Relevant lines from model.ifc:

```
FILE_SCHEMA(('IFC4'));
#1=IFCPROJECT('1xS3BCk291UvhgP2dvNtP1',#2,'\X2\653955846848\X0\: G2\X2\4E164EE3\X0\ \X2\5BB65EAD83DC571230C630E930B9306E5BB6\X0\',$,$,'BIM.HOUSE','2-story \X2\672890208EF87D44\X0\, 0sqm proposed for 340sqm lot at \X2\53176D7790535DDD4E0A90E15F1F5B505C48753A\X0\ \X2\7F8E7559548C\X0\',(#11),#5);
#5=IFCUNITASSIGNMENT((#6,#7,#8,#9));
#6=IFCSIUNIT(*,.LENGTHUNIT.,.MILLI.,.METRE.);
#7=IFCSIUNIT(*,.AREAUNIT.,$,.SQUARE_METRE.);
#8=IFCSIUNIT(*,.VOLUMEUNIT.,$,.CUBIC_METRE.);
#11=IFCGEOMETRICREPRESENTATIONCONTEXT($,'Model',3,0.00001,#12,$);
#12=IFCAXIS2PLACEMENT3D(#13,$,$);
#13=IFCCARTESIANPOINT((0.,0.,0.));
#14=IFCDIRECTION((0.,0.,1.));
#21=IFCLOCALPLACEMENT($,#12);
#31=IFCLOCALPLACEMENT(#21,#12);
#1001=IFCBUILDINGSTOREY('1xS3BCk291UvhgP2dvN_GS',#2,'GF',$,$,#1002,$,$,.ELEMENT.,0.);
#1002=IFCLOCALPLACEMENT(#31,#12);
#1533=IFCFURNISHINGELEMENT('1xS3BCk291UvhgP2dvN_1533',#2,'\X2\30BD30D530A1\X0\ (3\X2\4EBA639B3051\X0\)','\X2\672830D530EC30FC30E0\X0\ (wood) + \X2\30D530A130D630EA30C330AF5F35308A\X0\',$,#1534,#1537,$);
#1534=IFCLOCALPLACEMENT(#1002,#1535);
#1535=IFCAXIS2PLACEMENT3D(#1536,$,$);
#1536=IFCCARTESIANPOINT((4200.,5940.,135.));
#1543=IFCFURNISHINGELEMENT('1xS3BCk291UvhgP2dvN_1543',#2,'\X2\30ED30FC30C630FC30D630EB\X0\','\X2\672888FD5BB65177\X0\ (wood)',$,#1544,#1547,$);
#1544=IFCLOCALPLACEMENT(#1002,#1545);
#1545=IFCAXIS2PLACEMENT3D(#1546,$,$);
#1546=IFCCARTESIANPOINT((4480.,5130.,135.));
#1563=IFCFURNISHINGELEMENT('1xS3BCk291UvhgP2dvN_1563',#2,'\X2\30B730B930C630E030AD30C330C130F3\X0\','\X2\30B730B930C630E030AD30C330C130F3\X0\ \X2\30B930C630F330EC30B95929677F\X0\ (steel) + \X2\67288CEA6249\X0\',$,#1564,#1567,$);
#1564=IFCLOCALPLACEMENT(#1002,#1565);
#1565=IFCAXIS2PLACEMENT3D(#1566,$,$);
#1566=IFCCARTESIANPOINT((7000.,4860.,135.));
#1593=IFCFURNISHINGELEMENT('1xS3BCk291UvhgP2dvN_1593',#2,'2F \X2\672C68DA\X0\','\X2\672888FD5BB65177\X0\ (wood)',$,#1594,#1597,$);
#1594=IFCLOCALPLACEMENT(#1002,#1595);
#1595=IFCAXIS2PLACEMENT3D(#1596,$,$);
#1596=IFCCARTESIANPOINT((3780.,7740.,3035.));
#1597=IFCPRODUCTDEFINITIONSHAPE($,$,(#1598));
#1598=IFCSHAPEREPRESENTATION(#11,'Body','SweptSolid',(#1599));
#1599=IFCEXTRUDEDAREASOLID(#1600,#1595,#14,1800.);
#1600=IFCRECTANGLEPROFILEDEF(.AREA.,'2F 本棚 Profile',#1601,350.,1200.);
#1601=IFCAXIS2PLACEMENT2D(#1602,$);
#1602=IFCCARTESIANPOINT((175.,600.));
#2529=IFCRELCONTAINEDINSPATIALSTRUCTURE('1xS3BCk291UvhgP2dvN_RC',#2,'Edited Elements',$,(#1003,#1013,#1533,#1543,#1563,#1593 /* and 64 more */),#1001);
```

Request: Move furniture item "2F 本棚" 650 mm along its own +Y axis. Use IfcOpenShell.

```python
import ifcopenshell
import ifcopenshell.api.geometry
import ifcopenshell.util.placement
import ifcopenshell.util.unit

model = ifcopenshell.open("model.ifc")
unit_scale = ifcopenshell.util.unit.calculate_unit_scale(model)

item = model.by_guid("1xS3BCk291UvhgP2dvN_1593")
matrix = ifcopenshell.util.placement.get_local_placement(item.ObjectPlacement)
matrix[:3, 3] += matrix[:3, 1] * 0.65 / unit_scale
ifcopenshell.api.geometry.edit_object_placement(model, product=item, matrix=matrix, is_si=False)

print(ifcopenshell.util.placement.get_local_placement(item.ObjectPlacement).round(3) + 0.0)

model.write("model_updated.ifc")
```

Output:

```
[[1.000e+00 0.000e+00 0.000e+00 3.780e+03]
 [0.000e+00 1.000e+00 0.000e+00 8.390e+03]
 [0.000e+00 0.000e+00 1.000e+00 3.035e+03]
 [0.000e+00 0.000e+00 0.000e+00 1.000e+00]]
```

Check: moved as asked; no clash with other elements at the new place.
